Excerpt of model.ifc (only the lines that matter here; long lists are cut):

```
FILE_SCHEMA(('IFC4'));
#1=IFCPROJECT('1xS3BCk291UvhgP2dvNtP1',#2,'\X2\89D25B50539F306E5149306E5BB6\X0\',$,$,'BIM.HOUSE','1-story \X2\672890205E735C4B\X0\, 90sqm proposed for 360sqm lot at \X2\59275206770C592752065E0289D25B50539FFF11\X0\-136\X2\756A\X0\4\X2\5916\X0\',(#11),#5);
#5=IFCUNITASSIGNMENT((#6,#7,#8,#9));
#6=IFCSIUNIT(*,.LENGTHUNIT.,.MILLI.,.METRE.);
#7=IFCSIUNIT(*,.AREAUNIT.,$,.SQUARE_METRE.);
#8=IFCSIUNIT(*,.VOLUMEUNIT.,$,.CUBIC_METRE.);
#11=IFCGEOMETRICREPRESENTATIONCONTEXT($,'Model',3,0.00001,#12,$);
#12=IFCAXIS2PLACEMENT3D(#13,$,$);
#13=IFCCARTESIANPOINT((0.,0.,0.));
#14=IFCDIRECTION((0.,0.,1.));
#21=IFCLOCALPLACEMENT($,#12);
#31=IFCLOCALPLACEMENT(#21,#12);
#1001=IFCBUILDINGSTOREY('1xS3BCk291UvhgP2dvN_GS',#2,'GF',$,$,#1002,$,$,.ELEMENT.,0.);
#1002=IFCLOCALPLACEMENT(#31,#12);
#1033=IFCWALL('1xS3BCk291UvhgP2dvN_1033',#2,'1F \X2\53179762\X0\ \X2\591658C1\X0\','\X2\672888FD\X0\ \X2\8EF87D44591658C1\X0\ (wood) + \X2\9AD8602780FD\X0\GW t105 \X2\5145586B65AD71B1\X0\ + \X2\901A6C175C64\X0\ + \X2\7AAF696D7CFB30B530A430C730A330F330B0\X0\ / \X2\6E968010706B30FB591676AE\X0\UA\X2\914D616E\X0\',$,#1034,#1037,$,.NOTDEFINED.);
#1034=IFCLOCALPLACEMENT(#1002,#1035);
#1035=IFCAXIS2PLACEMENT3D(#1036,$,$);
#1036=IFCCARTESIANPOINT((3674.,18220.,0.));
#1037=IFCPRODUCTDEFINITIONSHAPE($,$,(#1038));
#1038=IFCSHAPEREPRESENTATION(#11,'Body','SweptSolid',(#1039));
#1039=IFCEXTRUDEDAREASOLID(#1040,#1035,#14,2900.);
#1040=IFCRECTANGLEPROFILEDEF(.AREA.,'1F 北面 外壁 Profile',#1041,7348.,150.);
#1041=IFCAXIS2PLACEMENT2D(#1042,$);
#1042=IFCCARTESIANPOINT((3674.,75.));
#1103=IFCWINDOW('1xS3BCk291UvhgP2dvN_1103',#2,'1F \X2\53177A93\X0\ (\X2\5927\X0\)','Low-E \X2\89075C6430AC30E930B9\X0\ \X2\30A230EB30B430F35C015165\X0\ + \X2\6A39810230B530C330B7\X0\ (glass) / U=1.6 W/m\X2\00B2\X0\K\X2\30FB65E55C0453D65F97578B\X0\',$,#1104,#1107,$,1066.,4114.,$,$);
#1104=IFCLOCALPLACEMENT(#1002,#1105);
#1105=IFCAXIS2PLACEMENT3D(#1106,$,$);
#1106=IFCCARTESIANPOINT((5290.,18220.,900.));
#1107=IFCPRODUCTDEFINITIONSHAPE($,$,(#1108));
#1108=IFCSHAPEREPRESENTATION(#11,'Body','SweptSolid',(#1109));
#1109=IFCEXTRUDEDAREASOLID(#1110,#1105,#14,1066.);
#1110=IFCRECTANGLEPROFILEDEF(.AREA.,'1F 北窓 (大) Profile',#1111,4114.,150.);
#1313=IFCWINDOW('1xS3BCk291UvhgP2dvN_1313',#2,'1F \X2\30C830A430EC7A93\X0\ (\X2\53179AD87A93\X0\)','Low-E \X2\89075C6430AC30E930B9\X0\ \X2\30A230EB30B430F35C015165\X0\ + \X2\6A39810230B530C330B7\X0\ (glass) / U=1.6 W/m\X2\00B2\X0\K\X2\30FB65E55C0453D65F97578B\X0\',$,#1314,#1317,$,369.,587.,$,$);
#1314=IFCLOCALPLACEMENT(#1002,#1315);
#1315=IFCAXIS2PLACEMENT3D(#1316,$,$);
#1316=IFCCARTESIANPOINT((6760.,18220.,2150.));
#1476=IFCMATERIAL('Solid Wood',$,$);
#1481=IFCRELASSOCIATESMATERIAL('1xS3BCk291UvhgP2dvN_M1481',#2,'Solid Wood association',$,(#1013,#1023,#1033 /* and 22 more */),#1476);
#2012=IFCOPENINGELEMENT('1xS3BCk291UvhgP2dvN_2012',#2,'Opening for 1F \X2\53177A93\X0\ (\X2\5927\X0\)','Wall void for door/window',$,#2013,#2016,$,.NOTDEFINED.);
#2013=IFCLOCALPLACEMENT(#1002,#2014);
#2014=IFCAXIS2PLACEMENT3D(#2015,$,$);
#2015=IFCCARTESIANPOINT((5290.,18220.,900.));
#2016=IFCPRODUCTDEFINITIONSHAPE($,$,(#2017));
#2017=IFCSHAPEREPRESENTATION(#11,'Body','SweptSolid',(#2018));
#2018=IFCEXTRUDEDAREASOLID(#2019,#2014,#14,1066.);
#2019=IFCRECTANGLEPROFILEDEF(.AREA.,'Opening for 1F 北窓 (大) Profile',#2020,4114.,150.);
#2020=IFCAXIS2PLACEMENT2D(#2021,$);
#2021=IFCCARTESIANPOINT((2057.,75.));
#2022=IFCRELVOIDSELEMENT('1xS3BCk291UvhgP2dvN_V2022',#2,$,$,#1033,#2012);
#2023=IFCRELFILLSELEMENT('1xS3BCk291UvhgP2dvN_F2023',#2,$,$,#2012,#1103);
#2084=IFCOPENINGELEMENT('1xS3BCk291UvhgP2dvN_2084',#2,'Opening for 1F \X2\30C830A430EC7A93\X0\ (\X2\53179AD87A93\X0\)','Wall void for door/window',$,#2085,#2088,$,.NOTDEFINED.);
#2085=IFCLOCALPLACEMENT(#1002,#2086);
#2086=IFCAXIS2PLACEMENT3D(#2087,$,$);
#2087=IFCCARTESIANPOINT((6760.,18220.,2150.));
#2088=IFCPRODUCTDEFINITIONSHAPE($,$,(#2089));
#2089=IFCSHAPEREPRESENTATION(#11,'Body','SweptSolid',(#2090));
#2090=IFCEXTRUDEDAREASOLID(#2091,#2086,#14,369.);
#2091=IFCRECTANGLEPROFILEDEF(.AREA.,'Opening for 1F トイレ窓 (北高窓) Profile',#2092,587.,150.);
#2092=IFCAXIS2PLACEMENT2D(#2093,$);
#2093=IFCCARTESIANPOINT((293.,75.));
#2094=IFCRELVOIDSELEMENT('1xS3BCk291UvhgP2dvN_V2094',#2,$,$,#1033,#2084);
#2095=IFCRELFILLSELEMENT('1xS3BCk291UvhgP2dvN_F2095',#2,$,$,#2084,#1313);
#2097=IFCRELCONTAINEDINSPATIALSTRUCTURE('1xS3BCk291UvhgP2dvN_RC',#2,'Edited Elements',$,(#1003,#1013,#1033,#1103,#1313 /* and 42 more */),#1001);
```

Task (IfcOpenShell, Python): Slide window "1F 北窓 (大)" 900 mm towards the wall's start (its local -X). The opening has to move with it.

```python
import ifcopenshell
import ifcopenshell.api.geometry
import ifcopenshell.util.placement
import ifcopenshell.util.unit

model = ifcopenshell.open("model.ifc")
unit_scale = ifcopenshell.util.unit.calculate_unit_scale(model)

window = model.by_guid("1xS3BCk291UvhgP2dvN_1103")
opening = window.FillsVoids[0].RelatingOpeningElement
wall = opening.VoidsElements[0].RelatingBuildingElement

wall_matrix = ifcopenshell.util.placement.get_local_placement(wall.ObjectPlacement)
shift = wall_matrix[:3, 0] * -0.9 / unit_scale
before = ifcopenshell.util.placement.get_local_placement(window.ObjectPlacement)[:3, 3].copy()

# The window is not placed relative to its opening, so move both.
for product in (opening, window):
    matrix = ifcopenshell.util.placement.get_local_placement(product.ObjectPlacement)
    matrix[:3, 3] += shift
    ifcopenshell.api.geometry.edit_object_placement(model, product=product, matrix=matrix, is_si=False)

after = ifcopenshell.util.placement.get_local_placement(window.ObjectPlacement)[:3, 3]
print("window moved by", (after - before).round(3) + 0.0)

model.write("model_v2.ifc")
```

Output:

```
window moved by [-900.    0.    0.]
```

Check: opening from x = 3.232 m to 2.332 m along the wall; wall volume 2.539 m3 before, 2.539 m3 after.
